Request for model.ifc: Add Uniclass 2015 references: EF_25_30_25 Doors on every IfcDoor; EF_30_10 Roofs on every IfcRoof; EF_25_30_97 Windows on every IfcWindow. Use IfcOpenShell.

First a look at what the model holds.

```python
import ifcopenshell

model = ifcopenshell.open("model.ifc")
print(model.schema)
print("classifications:", [c.Name for c in model.by_type("IfcClassification")])
for ifc_class in ("IfcDoor", "IfcRoof", "IfcStair", "IfcWall", "IfcWindow"):
    print(ifc_class, len(model.by_type(ifc_class)))
```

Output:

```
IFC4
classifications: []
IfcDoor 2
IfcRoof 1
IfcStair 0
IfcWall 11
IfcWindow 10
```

```python
import ifcopenshell
import ifcopenshell.api.classification

model = ifcopenshell.open("model.ifc")

system = ifcopenshell.api.classification.add_classification(model, classification="Uniclass 2015")

codes = {
    "IfcDoor": ("EF_25_30_25", "Doors"),
    "IfcRoof": ("EF_30_10", "Roofs"),
    "IfcWindow": ("EF_25_30_97", "Windows"),
}
for ifc_class, (code, name) in codes.items():
    products = model.by_type(ifc_class)
    ifcopenshell.api.classification.add_reference(
        model, products=products, classification=system, identification=code, name=name
    )
    print(code, len(products))

model.write("model_v2.ifc")
```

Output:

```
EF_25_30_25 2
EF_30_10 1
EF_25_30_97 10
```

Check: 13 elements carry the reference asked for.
